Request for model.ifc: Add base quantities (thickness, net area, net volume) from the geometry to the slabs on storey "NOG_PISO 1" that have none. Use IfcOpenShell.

First a look at what the model holds.

```python
import ifcopenshell
import ifcopenshell.util.element
import ifcopenshell.util.unit

model = ifcopenshell.open("model.ifc")
print(model.schema)
for unit_type in ("LENGTHUNIT", "AREAUNIT", "VOLUMEUNIT"):
    print(unit_type, ifcopenshell.util.unit.calculate_unit_scale(model, unit_type))
storey = next(s for s in model.by_type("IfcBuildingStorey") if s.Name == "NOG_PISO 1")
slabs = [e for e in ifcopenshell.util.element.get_decomposition(storey) if e.is_a("IfcSlab")]
for e in sorted(slabs, key=lambda e: e.id()):
    print(e.id(), e.is_a(), e.Name, list(ifcopenshell.util.element.get_psets(e, qtos_only=True)), sep=" | ")
```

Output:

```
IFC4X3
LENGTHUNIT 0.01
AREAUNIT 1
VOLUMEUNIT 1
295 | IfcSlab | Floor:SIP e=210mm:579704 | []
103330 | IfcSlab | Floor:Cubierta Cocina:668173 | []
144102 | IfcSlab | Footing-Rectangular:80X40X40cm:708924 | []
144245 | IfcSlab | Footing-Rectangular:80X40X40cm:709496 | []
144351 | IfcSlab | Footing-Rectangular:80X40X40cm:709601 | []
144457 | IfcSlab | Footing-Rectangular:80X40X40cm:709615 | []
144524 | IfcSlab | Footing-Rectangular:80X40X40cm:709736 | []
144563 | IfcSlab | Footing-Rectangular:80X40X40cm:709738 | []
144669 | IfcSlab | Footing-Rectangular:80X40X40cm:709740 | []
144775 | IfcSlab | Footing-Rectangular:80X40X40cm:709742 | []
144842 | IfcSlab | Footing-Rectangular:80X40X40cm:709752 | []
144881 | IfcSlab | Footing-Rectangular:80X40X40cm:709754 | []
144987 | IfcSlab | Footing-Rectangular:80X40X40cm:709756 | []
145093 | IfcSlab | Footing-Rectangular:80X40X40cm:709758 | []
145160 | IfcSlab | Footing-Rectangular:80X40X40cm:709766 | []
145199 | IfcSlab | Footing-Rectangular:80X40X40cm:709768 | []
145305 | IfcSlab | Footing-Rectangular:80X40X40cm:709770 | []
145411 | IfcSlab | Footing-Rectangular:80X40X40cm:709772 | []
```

```python
import ifcopenshell
import ifcopenshell.api.pset
import ifcopenshell.geom
import ifcopenshell.util.element
import ifcopenshell.util.shape
import ifcopenshell.util.unit

model = ifcopenshell.open("model.ifc")
unit_scale = ifcopenshell.util.unit.calculate_unit_scale(model)
area_scale = ifcopenshell.util.unit.calculate_unit_scale(model, "AREAUNIT")
volume_scale = ifcopenshell.util.unit.calculate_unit_scale(model, "VOLUMEUNIT")
settings = ifcopenshell.geom.settings()

storey = next(s for s in model.by_type("IfcBuildingStorey") if s.Name == "NOG_PISO 1")
slabs = [e for e in ifcopenshell.util.element.get_decomposition(storey) if e.is_a("IfcSlab")]

for e in sorted(slabs, key=lambda e: e.id()):
    if ifcopenshell.util.element.get_psets(e, qtos_only=True, should_inherit=False):
        continue
    # Geometry comes back in metres, in the element's own axes.
    shape = ifcopenshell.geom.create_shape(settings, e)
    values = {
        "Width": ifcopenshell.util.shape.get_z(shape.geometry) / unit_scale,
        "NetArea": ifcopenshell.util.shape.get_footprint_area(shape.geometry) / area_scale,
        "NetVolume": ifcopenshell.util.shape.get_volume(shape.geometry) / volume_scale,
    }
    qto = ifcopenshell.api.pset.add_qto(model, product=e, name="Qto_SlabBaseQuantities")
    ifcopenshell.api.pset.edit_qto(model, qto=qto, properties=values)
    print(e.id(), {k: round(v, 3) for k, v in values.items()})

model.write("model_updated.ifc")
```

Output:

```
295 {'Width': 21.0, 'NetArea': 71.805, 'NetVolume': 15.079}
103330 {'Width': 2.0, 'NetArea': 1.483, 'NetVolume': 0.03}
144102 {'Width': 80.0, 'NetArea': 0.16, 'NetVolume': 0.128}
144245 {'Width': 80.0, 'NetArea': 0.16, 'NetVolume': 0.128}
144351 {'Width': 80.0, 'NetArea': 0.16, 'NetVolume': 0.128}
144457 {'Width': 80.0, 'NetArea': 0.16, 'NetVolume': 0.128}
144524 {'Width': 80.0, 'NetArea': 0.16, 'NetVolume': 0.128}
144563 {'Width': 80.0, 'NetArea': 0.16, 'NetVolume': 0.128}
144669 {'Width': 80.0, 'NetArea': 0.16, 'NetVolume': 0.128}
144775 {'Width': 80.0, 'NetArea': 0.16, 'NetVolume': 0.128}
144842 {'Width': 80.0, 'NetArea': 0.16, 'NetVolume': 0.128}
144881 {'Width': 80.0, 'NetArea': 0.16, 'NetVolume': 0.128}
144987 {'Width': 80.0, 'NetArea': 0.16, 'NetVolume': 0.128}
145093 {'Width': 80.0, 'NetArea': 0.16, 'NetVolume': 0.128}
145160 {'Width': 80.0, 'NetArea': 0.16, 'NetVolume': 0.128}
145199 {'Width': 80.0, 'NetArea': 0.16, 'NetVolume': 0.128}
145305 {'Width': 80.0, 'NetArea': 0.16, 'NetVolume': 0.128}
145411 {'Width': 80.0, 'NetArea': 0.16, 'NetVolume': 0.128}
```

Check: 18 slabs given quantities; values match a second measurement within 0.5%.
